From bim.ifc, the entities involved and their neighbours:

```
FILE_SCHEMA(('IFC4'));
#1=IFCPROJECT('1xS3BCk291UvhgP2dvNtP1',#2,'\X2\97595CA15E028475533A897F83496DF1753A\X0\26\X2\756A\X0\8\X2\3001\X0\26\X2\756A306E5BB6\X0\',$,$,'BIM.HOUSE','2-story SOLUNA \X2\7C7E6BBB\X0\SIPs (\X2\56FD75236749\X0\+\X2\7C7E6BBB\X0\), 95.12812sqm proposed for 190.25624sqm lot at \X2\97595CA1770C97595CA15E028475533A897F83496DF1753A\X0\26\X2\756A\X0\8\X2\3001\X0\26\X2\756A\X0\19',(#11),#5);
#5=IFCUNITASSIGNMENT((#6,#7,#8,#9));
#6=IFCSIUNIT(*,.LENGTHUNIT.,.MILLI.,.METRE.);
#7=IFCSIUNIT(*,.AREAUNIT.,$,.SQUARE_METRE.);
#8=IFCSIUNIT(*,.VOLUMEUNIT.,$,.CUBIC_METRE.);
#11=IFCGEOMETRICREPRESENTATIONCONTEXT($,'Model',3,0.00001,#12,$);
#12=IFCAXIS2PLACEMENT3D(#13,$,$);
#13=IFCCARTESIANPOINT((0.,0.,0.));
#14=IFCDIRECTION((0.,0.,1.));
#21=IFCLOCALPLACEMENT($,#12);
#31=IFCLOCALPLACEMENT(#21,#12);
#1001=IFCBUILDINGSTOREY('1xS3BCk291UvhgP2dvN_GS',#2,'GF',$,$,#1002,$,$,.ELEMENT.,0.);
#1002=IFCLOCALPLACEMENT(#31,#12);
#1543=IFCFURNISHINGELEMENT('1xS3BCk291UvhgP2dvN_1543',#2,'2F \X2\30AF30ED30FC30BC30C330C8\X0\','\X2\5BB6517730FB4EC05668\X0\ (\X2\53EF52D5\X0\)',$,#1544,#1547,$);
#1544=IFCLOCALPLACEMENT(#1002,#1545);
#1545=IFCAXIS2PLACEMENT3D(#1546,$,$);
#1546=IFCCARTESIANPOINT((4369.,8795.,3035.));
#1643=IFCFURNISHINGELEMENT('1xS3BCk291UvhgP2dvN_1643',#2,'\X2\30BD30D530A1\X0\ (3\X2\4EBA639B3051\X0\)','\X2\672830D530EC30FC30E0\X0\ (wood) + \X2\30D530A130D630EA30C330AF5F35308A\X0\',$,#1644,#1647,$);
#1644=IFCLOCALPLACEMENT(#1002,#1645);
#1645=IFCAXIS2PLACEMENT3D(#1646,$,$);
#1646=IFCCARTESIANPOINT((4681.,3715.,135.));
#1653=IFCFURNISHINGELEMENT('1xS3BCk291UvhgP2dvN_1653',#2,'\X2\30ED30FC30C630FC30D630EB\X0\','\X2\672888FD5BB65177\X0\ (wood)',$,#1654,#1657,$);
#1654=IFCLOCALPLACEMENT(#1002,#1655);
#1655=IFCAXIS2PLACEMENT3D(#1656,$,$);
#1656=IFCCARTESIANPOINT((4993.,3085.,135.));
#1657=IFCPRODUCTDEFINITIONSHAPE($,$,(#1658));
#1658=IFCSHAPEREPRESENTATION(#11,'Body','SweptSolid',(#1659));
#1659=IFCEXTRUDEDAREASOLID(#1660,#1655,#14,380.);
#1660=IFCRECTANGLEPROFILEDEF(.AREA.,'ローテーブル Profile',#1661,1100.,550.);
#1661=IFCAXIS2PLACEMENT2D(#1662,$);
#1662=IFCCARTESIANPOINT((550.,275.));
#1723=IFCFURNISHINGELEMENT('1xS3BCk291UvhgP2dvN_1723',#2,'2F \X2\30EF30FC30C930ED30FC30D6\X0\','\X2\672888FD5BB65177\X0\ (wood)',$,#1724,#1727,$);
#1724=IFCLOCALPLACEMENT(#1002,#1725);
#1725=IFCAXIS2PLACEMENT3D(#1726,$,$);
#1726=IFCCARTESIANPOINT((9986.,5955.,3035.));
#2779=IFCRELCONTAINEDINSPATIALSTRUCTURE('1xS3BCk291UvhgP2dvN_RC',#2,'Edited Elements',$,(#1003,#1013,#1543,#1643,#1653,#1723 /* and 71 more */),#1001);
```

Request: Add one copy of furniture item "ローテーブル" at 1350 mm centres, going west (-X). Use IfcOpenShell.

```python
import numpy as np
import ifcopenshell
import ifcopenshell.api.geometry
import ifcopenshell.api.root
import ifcopenshell.util.element
import ifcopenshell.util.placement

model = ifcopenshell.open("bim.ifc")


def reuse_history(source, copy):
    """copy_class also copies each property set's owner history, people and application; keep the originals."""
    for rel in copy.IsDefinedBy:
        if rel.is_a("IfcRelDefinesByProperties") and (history := rel.RelatingPropertyDefinition.OwnerHistory):
            rel.RelatingPropertyDefinition.OwnerHistory = source.OwnerHistory
            ifcopenshell.util.element.remove_deep2(model, history)


source = model.by_guid("1xS3BCk291UvhgP2dvN_1653")
base = ifcopenshell.util.placement.get_local_placement(source.ObjectPlacement)
step = np.array([-1.0, 0.0, 0.0]) * 1350.0

for i in range(1, 2):
    copy = ifcopenshell.api.root.copy_class(model, product=source)
    copy.Representation = ifcopenshell.util.element.copy_deep(
        model, source.Representation, exclude=["IfcGeometricRepresentationContext", "IfcRepresentationMap"]
    )
    reuse_history(source, copy)
    matrix = base.copy()
    matrix[:3, 3] += i * step
    print("added at", matrix[:3, 3].round(3) + 0.0)
    ifcopenshell.api.geometry.edit_object_placement(model, product=copy, matrix=matrix, is_si=False)

model.write("bim_updated.ifc")
```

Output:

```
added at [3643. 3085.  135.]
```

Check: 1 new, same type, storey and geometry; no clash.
